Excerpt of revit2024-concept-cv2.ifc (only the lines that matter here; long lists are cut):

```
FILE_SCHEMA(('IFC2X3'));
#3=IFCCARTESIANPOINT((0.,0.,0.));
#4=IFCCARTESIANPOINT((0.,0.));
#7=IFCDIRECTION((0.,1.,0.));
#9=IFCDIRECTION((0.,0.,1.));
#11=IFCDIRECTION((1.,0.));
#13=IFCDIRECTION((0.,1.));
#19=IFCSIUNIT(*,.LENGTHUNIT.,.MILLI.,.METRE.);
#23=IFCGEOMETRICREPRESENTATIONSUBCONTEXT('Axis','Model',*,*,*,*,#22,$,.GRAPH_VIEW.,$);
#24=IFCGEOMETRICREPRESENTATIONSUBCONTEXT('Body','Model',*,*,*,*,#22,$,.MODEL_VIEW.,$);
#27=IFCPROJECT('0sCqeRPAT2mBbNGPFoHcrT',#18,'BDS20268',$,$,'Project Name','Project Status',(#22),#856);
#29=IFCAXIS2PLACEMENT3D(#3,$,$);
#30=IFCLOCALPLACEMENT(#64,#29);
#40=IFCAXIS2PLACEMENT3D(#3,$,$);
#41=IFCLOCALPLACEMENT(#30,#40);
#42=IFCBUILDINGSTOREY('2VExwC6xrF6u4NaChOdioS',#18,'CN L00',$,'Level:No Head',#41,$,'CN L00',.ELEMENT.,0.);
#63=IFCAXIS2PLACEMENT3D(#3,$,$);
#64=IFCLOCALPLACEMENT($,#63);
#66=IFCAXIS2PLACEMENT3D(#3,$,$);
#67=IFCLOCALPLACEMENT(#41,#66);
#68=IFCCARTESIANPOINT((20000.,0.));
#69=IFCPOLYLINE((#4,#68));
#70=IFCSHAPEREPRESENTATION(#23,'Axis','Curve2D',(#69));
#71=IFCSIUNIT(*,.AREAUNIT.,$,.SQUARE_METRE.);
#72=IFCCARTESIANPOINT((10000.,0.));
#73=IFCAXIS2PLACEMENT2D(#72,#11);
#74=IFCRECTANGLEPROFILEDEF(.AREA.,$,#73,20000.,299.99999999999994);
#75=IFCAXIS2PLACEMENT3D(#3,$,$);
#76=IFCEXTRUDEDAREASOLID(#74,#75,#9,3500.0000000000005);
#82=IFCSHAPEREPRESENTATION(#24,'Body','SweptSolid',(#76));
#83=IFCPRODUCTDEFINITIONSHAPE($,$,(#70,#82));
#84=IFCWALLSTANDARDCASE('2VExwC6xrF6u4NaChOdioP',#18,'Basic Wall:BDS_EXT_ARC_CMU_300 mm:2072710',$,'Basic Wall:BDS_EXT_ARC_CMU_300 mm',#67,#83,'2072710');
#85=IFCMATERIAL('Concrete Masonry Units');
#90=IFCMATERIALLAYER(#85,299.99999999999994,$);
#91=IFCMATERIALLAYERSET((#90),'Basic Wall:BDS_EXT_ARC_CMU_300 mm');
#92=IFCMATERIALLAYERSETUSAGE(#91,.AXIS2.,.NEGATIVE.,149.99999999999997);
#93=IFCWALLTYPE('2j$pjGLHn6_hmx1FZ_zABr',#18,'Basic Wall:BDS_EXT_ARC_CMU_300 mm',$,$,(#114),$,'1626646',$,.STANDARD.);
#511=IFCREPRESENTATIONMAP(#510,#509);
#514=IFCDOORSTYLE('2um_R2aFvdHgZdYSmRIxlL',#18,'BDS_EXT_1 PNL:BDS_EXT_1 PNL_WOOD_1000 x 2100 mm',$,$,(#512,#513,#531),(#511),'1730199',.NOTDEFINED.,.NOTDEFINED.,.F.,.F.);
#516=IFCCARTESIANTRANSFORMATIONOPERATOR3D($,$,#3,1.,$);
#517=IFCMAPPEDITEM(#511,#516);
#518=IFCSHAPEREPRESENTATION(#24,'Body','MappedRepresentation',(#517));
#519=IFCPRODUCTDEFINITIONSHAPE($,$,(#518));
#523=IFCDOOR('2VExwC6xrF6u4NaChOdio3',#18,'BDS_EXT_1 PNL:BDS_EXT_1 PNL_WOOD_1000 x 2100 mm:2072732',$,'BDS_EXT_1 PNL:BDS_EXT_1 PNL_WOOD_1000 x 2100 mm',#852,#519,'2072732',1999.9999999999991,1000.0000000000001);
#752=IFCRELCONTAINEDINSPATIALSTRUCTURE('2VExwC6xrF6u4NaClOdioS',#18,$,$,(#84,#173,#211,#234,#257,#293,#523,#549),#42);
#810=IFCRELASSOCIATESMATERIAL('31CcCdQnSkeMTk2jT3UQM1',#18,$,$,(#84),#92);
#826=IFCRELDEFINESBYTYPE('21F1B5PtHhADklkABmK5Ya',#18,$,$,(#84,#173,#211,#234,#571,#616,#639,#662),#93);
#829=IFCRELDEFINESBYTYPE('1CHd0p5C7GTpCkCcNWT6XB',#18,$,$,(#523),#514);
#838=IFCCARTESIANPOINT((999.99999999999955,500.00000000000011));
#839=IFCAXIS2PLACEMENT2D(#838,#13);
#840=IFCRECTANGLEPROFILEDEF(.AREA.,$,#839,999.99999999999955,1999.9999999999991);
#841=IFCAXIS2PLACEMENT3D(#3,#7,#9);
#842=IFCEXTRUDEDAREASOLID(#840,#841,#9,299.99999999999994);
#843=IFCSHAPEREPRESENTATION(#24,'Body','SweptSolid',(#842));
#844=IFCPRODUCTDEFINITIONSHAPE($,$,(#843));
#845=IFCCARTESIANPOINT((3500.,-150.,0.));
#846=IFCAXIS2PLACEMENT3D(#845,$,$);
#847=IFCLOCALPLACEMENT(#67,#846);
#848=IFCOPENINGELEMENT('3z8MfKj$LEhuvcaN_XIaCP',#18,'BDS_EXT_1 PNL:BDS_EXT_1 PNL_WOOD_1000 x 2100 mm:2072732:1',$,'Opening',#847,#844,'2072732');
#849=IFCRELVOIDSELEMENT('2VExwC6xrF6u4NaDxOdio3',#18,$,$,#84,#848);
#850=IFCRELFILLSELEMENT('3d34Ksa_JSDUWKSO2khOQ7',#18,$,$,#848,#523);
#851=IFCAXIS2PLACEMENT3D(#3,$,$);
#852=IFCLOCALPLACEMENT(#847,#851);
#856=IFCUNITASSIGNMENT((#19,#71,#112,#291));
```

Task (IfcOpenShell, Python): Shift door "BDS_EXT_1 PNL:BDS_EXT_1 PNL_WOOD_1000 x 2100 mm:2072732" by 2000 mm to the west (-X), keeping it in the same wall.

```python
import ifcopenshell
import ifcopenshell.api.geometry
import ifcopenshell.util.placement

model = ifcopenshell.open("revit2024-concept-cv2.ifc")

door = model.by_id(523)
opening = door.FillsVoids[0].RelatingOpeningElement
wall = opening.VoidsElements[0].RelatingBuildingElement

wall_matrix = ifcopenshell.util.placement.get_local_placement(wall.ObjectPlacement)
shift = wall_matrix[:3, 0] * -2000.0
before = ifcopenshell.util.placement.get_local_placement(door.ObjectPlacement)[:3, 3].copy()

# The door is placed relative to its opening, so it follows when the opening moves.
matrix = ifcopenshell.util.placement.get_local_placement(opening.ObjectPlacement)
matrix[:3, 3] += shift
ifcopenshell.api.geometry.edit_object_placement(
    model, product=opening, matrix=matrix, is_si=False, should_transform_children=True
)

after = ifcopenshell.util.placement.get_local_placement(door.ObjectPlacement)[:3, 3]
print("door moved by", (after - before).round(3) + 0.0)

model.write("revit2024-concept-cv2_rev.ifc")
```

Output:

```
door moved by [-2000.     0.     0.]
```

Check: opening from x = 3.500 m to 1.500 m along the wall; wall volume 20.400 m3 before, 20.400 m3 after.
